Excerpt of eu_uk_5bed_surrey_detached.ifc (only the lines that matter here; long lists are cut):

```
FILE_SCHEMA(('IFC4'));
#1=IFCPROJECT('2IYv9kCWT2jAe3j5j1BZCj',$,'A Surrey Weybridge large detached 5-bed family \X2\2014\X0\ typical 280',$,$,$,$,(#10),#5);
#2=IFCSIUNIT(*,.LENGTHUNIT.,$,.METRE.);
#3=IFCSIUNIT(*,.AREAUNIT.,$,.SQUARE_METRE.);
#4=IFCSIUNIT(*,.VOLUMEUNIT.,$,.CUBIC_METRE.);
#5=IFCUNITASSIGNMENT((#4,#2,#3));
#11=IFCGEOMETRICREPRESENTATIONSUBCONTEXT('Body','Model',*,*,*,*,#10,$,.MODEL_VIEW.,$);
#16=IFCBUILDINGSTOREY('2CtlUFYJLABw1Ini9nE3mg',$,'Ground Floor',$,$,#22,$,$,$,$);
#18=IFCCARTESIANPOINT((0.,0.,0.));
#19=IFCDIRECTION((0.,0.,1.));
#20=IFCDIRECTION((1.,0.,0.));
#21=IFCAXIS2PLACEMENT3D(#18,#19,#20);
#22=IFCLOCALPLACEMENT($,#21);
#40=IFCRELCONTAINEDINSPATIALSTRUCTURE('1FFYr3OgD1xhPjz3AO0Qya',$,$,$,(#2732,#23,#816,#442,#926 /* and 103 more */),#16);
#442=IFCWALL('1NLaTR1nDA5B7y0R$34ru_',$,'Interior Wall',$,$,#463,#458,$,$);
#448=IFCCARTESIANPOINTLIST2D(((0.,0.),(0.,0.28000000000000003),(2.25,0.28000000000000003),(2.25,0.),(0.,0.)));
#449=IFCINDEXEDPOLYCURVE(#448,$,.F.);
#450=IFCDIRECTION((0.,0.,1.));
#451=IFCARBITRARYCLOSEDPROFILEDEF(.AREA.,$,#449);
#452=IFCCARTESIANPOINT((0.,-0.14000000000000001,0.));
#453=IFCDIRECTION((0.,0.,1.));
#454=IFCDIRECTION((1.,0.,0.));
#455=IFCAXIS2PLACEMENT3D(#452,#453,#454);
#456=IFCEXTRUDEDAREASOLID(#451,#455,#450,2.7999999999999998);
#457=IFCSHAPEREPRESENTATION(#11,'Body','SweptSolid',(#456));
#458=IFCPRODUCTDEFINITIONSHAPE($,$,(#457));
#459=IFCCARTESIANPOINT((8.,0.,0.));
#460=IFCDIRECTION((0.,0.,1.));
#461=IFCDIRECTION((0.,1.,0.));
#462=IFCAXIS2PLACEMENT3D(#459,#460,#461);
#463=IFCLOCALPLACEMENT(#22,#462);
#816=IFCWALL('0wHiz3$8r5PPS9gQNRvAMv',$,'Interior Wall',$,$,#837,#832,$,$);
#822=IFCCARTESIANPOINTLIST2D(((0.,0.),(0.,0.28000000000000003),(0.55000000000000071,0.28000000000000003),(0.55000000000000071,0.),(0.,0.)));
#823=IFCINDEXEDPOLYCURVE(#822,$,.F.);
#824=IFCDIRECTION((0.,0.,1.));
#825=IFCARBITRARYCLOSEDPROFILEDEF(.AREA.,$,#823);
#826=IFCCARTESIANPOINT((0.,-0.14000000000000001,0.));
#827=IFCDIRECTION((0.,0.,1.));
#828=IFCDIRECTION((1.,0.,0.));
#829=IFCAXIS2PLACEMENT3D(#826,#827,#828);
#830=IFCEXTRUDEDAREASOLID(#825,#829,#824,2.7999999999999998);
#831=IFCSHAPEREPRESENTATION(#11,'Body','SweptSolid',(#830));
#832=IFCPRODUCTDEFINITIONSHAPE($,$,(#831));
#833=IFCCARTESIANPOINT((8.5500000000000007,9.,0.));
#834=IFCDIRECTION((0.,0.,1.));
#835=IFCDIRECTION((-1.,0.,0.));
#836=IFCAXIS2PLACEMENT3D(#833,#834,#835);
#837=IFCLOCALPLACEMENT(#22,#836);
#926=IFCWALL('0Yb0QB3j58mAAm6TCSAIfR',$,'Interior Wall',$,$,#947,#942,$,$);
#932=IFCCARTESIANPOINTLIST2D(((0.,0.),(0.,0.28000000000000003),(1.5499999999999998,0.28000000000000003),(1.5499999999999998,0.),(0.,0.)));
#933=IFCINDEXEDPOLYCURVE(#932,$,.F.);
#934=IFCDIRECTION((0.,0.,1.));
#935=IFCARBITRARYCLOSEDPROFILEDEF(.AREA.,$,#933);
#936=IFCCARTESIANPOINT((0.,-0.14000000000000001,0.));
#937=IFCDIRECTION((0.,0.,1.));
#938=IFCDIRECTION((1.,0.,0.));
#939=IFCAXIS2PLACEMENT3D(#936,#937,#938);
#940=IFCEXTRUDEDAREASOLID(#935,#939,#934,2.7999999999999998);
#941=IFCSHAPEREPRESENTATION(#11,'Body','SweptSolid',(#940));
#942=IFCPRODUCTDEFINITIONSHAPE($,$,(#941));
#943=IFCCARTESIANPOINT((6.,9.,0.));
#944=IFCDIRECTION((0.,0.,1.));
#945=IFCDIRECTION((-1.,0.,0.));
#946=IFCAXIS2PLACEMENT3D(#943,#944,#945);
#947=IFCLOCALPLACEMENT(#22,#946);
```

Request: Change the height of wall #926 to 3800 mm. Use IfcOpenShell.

```python
import ifcopenshell
import ifcopenshell.geom
import ifcopenshell.util.representation
import ifcopenshell.util.shape

model = ifcopenshell.open("eu_uk_5bed_surrey_detached.ifc")
settings = ifcopenshell.geom.settings()


def volume(element):
    """Net volume in cubic metres, openings subtracted."""
    shape = ifcopenshell.geom.create_shape(settings, element)
    return ifcopenshell.util.shape.get_volume(shape.geometry)


wall = model.by_id(926)
before = volume(wall)

body = ifcopenshell.util.representation.get_representation(wall, "Model", "Body")
solid = body.Items[0]
old_height = solid.Depth
solid.Depth = 3.8
after = volume(wall)

print(f"height {old_height:g} -> {solid.Depth:g}, volume {before:.3f} -> {after:.3f} m3")

model.write("eu_uk_5bed_surrey_detached_v2.ifc")
```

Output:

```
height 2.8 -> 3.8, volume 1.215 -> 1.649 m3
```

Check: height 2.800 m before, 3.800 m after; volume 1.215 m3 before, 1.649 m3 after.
